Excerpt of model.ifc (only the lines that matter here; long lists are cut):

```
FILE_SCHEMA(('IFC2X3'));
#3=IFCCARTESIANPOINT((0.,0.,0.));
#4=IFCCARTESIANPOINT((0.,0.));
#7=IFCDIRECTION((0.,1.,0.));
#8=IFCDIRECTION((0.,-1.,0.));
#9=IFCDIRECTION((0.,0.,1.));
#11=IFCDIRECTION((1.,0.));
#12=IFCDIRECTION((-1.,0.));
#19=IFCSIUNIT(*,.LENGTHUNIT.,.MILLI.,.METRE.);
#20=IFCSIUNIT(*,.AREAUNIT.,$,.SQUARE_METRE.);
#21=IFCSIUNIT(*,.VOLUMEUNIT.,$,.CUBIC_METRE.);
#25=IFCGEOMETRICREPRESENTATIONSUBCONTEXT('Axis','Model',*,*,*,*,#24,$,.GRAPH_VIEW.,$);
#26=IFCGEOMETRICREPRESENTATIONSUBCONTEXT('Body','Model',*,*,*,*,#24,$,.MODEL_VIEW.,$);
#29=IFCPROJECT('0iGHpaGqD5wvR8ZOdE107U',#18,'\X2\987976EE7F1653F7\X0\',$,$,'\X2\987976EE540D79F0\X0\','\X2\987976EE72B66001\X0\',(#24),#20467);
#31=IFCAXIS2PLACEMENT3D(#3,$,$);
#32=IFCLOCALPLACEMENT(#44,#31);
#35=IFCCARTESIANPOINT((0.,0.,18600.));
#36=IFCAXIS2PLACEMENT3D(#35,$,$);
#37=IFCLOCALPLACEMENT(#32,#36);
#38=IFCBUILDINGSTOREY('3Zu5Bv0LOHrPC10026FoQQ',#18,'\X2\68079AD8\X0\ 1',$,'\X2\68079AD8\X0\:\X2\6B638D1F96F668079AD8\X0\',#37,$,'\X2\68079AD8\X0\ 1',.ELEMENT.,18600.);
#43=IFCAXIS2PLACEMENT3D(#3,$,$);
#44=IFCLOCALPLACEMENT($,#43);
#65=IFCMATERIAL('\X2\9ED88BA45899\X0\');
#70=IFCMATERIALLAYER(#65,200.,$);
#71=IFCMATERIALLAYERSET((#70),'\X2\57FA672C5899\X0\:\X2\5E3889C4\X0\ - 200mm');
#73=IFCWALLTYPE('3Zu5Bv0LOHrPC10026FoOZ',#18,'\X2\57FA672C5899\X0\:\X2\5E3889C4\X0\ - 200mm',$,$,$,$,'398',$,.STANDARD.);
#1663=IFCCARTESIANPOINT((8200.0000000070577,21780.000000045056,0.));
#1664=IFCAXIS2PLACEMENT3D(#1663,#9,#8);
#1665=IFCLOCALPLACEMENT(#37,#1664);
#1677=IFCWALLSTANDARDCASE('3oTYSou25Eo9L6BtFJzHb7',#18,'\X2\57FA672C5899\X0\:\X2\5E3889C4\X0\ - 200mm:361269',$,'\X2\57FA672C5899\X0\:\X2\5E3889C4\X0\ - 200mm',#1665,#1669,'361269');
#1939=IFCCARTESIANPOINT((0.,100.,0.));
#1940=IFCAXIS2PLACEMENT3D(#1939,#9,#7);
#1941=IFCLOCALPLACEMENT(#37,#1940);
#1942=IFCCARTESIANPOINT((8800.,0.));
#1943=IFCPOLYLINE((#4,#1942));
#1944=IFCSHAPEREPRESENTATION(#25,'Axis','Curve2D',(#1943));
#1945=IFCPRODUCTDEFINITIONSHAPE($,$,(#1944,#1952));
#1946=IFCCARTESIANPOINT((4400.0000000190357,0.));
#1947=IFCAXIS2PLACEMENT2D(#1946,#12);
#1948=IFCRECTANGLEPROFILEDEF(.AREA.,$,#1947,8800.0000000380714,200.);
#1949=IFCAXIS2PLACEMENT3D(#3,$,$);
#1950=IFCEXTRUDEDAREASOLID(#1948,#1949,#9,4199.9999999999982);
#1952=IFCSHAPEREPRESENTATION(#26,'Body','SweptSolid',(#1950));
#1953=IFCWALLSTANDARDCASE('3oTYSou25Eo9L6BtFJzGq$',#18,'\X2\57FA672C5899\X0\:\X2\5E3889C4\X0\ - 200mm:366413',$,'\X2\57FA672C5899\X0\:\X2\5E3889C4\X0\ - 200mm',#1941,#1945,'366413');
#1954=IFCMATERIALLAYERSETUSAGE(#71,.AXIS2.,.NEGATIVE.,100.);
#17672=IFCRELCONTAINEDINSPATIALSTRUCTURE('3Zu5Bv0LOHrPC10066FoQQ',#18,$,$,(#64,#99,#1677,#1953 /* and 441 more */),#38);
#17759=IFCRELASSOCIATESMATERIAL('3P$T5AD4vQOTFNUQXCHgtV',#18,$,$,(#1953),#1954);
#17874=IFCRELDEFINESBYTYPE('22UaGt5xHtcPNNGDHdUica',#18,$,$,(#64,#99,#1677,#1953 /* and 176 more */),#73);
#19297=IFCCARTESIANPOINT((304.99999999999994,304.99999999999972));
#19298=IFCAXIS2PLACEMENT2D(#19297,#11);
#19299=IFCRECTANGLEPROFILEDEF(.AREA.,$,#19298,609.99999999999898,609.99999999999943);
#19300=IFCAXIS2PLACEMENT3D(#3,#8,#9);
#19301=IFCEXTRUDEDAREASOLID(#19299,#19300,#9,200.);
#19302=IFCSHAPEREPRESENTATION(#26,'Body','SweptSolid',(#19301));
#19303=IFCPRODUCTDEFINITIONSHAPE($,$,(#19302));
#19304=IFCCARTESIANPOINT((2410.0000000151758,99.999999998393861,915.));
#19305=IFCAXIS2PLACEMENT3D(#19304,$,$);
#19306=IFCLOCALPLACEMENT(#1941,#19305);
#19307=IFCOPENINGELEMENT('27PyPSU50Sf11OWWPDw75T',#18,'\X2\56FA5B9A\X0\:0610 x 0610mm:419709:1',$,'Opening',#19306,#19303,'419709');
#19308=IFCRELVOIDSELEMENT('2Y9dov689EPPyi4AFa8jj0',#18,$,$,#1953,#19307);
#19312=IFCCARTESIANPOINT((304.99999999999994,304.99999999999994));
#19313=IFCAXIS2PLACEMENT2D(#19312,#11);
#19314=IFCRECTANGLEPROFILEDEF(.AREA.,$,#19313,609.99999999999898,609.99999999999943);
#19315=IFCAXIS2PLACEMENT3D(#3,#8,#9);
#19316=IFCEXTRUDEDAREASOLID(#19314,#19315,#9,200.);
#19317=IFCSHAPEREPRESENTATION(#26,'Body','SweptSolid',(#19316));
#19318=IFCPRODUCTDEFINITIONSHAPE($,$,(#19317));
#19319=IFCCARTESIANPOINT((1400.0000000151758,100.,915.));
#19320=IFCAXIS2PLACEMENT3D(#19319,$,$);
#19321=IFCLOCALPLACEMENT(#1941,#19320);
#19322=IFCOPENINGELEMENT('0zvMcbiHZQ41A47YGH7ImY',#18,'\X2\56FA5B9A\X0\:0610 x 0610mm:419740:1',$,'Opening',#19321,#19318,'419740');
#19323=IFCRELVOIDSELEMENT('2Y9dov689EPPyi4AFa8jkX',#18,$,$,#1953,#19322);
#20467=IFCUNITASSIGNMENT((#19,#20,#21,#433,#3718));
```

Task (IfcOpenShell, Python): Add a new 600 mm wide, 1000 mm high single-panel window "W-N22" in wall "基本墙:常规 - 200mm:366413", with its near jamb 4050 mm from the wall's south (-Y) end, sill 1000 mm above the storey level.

```python
import numpy as np
import ifcopenshell
import ifcopenshell.api.feature
import ifcopenshell.api.geometry
import ifcopenshell.api.root
import ifcopenshell.api.spatial
import ifcopenshell.api.type
import ifcopenshell.geom
import ifcopenshell.util.element
import ifcopenshell.util.placement
import ifcopenshell.util.representation
import ifcopenshell.util.shape
import ifcopenshell.util.unit

model = ifcopenshell.open("model.ifc")
unit_scale = ifcopenshell.util.unit.calculate_unit_scale(model)
settings = ifcopenshell.geom.settings()


def volume(element):
    """Net volume in cubic metres, openings subtracted."""
    shape = ifcopenshell.geom.create_shape(settings, element)
    return ifcopenshell.util.shape.get_volume(shape.geometry)


wall = model.by_id(1953)
storey = ifcopenshell.util.element.get_container(wall, ifc_class="IfcBuildingStorey")
context = ifcopenshell.util.representation.get_context(model, "Model", "Body", "MODEL_VIEW")
before = volume(wall)

width, height, from_end, sill = 0.6, 1, 4.05, 1  # metres

# The wall runs along its own X axis, and the end named is its -X end.
wall_shape = ifcopenshell.geom.create_shape(settings, wall)
x, y, z = ifcopenshell.util.shape.get_vertices(wall_shape.geometry).T
start = x.min() + from_end
face, thickness = float(y.min()), float(y.max() - y.min())
wall_matrix = ifcopenshell.util.placement.get_local_placement(wall.ObjectPlacement)
level = ifcopenshell.util.placement.get_local_placement(storey.ObjectPlacement)[2, 3]


def in_wall(x, y):
    """Placement at x, y metres in the wall's axes, at sill height."""
    matrix = wall_matrix.copy()
    matrix[:, 3] = wall_matrix @ np.array([x / unit_scale, y / unit_scale, 0.0, 1.0])
    matrix[2, 3] = level + sill / unit_scale
    return matrix


# Opening: a box that overshoots both wall faces by 50 mm.
opening = ifcopenshell.api.root.create_entity(model, ifc_class="IfcOpeningElement")
box = ifcopenshell.api.geometry.add_wall_representation(
    model, context=context, length=width, height=height, thickness=thickness + 0.1
)
ifcopenshell.api.geometry.assign_representation(model, product=opening, representation=box)
ifcopenshell.api.geometry.edit_object_placement(model, product=opening, matrix=in_wall(start, face - 0.05), is_si=False)
ifcopenshell.api.feature.add_feature(model, feature=opening, element=wall)

window = ifcopenshell.api.root.create_entity(model, ifc_class="IfcWindow", name="W-N22")
window.OverallWidth, window.OverallHeight = width / unit_scale, height / unit_scale
body = ifcopenshell.api.geometry.add_window_representation(
    model,
    context=context,
    overall_width=window.OverallWidth,
    overall_height=window.OverallHeight,
    partition_type="SINGLE_PANEL",
)
ifcopenshell.api.geometry.assign_representation(model, product=window, representation=body)
ifcopenshell.api.spatial.assign_container(model, products=[window], relating_structure=storey)
fills = ifcopenshell.api.feature.add_filling(model, opening=opening, element=window)
fills.OwnerHistory = window.OwnerHistory  # required in IFC2X3

# IFC2X3 keeps the operation on the window style.
style = ifcopenshell.api.root.create_entity(model, ifc_class="IfcWindowStyle", name="W-N22")
style.OperationType, style.ConstructionType = "SINGLE_PANEL", "NOTDEFINED"
style.ParameterTakesPrecedence = style.Sizeable = False
ifcopenshell.api.type.assign_type(model, related_objects=[window], relating_type=style)

# Centre the window in the wall's thickness.
ifcopenshell.api.geometry.edit_object_placement(model, product=window, matrix=in_wall(start, face), is_si=False)
window_shape = ifcopenshell.geom.create_shape(settings, window)
depth = ifcopenshell.util.shape.get_vertices(window_shape.geometry)[:, 1]
offset = face + thickness / 2 - (depth.min() + depth.max()) / 2
ifcopenshell.api.geometry.edit_object_placement(model, product=window, matrix=in_wall(start, offset), is_si=False)

after = volume(wall)

print(f"wall volume {before:.3f} -> {after:.3f} m3")

model.write("model-out.ifc")
```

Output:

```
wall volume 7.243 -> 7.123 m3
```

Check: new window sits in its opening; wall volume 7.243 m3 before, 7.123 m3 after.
